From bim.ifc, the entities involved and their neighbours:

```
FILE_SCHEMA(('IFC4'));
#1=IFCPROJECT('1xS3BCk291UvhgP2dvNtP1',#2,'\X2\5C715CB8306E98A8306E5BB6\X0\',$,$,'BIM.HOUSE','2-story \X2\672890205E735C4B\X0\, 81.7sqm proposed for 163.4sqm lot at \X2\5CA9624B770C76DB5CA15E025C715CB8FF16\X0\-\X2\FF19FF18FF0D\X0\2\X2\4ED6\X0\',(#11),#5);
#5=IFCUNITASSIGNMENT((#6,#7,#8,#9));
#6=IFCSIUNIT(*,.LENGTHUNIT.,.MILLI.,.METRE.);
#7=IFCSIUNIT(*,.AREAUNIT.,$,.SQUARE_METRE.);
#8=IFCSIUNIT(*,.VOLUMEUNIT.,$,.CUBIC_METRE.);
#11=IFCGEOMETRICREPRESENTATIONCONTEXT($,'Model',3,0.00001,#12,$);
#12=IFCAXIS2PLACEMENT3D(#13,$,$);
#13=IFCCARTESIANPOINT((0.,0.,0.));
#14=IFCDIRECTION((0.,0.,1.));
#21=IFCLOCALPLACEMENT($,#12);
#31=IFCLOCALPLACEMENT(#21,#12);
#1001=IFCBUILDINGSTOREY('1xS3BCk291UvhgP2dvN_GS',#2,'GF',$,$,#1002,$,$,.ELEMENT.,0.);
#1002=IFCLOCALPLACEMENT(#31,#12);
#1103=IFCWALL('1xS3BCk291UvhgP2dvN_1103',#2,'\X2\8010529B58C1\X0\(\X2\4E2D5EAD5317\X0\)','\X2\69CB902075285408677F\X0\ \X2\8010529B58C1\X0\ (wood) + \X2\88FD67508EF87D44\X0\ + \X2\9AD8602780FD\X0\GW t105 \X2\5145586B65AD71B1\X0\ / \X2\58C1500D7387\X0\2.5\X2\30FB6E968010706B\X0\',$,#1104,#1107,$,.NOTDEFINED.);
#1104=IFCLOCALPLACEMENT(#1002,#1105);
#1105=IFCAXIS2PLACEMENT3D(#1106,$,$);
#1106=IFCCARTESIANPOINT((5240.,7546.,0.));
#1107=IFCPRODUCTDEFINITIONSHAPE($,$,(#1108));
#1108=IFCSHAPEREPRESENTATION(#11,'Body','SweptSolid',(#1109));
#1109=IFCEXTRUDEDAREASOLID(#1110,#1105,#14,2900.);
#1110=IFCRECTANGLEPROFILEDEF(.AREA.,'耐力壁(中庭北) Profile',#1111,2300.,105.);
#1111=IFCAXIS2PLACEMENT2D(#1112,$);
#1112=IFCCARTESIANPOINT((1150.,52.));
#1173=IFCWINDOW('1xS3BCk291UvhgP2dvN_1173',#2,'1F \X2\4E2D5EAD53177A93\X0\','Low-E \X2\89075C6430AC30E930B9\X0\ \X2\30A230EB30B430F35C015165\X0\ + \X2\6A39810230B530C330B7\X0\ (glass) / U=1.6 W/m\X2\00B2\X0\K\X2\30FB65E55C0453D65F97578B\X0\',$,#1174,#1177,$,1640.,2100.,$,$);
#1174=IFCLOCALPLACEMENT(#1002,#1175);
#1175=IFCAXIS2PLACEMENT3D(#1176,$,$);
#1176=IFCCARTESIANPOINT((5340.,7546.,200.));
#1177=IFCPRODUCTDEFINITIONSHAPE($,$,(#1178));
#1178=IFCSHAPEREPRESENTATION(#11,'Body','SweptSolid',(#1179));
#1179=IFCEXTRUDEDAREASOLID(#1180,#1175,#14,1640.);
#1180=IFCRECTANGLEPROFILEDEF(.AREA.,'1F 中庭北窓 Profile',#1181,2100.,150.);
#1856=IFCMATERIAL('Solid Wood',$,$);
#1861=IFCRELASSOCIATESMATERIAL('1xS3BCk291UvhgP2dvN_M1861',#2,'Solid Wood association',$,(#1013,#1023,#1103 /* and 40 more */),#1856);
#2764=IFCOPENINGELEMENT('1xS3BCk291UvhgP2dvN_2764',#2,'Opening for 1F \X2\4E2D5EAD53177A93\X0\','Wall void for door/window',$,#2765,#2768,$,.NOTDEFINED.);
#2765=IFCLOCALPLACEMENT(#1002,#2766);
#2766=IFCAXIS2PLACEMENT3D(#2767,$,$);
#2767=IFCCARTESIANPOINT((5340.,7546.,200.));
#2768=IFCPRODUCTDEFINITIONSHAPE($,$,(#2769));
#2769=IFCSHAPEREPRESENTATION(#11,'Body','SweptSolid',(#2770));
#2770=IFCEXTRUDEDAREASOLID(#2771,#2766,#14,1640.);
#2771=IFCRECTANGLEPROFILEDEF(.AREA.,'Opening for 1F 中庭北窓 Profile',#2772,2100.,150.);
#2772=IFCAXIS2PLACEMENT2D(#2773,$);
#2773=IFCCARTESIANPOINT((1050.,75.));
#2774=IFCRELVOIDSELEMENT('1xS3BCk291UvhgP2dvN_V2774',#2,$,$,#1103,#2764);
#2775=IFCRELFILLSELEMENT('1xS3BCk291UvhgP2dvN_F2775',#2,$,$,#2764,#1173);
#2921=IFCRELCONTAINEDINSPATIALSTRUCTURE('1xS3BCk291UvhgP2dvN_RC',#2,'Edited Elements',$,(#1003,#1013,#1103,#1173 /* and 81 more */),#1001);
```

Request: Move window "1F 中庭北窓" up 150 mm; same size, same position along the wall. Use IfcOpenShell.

```python
import numpy as np
import ifcopenshell
import ifcopenshell.api.geometry
import ifcopenshell.util.placement
import ifcopenshell.util.unit

model = ifcopenshell.open("bim.ifc")
unit_scale = ifcopenshell.util.unit.calculate_unit_scale(model)

window = model.by_guid("1xS3BCk291UvhgP2dvN_1173")
opening = window.FillsVoids[0].RelatingOpeningElement
dz = 150.0

shift = np.array([0.0, 0.0, dz])
# The window is not placed relative to its opening, so move both.
for product in (opening, window):
    matrix = ifcopenshell.util.placement.get_local_placement(product.ObjectPlacement)
    matrix[:3, 3] += shift
    ifcopenshell.api.geometry.edit_object_placement(model, product=product, matrix=matrix, is_si=False)

print(f"moved by {dz * unit_scale:+.3f} m")

model.write("bim-out.ifc")
```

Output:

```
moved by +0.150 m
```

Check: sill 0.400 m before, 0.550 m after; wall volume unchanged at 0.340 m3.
